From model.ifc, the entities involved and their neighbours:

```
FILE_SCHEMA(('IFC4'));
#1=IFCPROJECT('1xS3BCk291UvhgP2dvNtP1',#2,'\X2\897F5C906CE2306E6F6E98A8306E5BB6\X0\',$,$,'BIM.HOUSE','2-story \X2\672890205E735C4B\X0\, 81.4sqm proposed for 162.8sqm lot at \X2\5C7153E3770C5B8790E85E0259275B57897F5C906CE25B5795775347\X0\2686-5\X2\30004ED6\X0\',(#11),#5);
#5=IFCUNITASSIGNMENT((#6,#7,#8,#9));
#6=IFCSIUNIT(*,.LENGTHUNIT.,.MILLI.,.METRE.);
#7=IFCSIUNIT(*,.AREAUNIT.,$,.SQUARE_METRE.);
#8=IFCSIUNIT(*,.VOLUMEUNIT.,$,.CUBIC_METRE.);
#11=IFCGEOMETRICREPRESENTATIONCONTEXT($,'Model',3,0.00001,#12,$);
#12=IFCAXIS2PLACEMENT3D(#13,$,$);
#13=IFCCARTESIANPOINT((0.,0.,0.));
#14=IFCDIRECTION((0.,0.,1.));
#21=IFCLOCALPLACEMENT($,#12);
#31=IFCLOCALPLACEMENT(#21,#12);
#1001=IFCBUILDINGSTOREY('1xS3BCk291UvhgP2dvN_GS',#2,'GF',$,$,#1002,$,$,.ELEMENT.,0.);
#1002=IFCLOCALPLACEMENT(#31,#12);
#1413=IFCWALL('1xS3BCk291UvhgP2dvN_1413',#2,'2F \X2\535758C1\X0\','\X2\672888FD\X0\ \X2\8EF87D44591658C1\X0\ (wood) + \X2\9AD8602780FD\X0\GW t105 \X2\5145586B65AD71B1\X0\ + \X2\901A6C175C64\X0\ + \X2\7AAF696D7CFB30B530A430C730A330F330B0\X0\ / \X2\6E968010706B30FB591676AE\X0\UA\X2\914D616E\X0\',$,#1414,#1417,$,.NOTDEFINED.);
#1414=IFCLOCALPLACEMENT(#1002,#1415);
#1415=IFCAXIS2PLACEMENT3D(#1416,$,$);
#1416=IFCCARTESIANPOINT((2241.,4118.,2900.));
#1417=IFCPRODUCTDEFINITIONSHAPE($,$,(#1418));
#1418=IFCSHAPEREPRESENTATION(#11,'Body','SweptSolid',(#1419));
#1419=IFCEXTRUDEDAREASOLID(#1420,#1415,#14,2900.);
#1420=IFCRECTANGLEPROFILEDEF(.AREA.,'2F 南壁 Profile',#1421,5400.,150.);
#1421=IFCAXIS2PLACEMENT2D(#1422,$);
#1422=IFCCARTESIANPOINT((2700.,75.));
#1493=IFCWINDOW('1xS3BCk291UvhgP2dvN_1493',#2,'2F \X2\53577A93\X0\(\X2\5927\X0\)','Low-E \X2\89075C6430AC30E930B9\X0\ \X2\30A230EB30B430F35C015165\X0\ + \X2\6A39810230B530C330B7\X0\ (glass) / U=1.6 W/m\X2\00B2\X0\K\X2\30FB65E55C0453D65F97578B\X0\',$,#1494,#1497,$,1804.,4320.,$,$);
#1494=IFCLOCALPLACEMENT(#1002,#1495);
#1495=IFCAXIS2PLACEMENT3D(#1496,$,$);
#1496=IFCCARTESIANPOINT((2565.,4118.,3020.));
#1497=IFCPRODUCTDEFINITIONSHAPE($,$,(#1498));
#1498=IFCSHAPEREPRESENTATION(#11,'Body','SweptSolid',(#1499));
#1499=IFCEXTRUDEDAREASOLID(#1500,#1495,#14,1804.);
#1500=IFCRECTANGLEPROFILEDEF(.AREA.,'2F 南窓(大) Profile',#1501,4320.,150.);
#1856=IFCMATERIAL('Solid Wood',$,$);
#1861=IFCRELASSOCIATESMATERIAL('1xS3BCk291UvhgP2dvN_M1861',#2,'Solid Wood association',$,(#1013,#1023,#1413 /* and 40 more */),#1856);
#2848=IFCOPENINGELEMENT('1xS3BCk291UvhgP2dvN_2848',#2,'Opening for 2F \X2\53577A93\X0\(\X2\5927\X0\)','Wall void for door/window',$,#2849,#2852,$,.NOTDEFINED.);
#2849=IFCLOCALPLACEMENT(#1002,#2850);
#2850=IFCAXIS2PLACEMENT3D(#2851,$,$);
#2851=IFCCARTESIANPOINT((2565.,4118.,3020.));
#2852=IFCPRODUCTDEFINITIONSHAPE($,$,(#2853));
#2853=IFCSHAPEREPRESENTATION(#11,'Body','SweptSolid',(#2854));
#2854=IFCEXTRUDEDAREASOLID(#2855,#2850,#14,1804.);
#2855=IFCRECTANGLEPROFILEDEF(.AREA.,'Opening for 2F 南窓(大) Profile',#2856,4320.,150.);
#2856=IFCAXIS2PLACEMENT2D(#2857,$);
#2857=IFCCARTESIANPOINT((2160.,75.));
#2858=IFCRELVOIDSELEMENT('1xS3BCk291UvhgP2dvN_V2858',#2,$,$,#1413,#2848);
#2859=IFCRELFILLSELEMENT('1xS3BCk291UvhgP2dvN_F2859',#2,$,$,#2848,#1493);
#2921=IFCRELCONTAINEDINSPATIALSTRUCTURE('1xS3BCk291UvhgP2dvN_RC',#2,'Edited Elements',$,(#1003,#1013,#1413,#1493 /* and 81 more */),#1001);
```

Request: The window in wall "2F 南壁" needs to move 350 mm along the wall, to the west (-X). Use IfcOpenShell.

```python
import ifcopenshell
import ifcopenshell.api.geometry
import ifcopenshell.util.placement
import ifcopenshell.util.unit

model = ifcopenshell.open("model.ifc")
unit_scale = ifcopenshell.util.unit.calculate_unit_scale(model)

window = model.by_guid("1xS3BCk291UvhgP2dvN_1493")
opening = window.FillsVoids[0].RelatingOpeningElement
wall = opening.VoidsElements[0].RelatingBuildingElement

wall_matrix = ifcopenshell.util.placement.get_local_placement(wall.ObjectPlacement)
shift = wall_matrix[:3, 0] * -0.35 / unit_scale
before = ifcopenshell.util.placement.get_local_placement(window.ObjectPlacement)[:3, 3].copy()

# The window is not placed relative to its opening, so move both.
for product in (opening, window):
    matrix = ifcopenshell.util.placement.get_local_placement(product.ObjectPlacement)
    matrix[:3, 3] += shift
    ifcopenshell.api.geometry.edit_object_placement(model, product=product, matrix=matrix, is_si=False)

after = ifcopenshell.util.placement.get_local_placement(window.ObjectPlacement)[:3, 3]
print("window moved by", (after - before).round(3) + 0.0)

model.write("model_rev.ifc")
```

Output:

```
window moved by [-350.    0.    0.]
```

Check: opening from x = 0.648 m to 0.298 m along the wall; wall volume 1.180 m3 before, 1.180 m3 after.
